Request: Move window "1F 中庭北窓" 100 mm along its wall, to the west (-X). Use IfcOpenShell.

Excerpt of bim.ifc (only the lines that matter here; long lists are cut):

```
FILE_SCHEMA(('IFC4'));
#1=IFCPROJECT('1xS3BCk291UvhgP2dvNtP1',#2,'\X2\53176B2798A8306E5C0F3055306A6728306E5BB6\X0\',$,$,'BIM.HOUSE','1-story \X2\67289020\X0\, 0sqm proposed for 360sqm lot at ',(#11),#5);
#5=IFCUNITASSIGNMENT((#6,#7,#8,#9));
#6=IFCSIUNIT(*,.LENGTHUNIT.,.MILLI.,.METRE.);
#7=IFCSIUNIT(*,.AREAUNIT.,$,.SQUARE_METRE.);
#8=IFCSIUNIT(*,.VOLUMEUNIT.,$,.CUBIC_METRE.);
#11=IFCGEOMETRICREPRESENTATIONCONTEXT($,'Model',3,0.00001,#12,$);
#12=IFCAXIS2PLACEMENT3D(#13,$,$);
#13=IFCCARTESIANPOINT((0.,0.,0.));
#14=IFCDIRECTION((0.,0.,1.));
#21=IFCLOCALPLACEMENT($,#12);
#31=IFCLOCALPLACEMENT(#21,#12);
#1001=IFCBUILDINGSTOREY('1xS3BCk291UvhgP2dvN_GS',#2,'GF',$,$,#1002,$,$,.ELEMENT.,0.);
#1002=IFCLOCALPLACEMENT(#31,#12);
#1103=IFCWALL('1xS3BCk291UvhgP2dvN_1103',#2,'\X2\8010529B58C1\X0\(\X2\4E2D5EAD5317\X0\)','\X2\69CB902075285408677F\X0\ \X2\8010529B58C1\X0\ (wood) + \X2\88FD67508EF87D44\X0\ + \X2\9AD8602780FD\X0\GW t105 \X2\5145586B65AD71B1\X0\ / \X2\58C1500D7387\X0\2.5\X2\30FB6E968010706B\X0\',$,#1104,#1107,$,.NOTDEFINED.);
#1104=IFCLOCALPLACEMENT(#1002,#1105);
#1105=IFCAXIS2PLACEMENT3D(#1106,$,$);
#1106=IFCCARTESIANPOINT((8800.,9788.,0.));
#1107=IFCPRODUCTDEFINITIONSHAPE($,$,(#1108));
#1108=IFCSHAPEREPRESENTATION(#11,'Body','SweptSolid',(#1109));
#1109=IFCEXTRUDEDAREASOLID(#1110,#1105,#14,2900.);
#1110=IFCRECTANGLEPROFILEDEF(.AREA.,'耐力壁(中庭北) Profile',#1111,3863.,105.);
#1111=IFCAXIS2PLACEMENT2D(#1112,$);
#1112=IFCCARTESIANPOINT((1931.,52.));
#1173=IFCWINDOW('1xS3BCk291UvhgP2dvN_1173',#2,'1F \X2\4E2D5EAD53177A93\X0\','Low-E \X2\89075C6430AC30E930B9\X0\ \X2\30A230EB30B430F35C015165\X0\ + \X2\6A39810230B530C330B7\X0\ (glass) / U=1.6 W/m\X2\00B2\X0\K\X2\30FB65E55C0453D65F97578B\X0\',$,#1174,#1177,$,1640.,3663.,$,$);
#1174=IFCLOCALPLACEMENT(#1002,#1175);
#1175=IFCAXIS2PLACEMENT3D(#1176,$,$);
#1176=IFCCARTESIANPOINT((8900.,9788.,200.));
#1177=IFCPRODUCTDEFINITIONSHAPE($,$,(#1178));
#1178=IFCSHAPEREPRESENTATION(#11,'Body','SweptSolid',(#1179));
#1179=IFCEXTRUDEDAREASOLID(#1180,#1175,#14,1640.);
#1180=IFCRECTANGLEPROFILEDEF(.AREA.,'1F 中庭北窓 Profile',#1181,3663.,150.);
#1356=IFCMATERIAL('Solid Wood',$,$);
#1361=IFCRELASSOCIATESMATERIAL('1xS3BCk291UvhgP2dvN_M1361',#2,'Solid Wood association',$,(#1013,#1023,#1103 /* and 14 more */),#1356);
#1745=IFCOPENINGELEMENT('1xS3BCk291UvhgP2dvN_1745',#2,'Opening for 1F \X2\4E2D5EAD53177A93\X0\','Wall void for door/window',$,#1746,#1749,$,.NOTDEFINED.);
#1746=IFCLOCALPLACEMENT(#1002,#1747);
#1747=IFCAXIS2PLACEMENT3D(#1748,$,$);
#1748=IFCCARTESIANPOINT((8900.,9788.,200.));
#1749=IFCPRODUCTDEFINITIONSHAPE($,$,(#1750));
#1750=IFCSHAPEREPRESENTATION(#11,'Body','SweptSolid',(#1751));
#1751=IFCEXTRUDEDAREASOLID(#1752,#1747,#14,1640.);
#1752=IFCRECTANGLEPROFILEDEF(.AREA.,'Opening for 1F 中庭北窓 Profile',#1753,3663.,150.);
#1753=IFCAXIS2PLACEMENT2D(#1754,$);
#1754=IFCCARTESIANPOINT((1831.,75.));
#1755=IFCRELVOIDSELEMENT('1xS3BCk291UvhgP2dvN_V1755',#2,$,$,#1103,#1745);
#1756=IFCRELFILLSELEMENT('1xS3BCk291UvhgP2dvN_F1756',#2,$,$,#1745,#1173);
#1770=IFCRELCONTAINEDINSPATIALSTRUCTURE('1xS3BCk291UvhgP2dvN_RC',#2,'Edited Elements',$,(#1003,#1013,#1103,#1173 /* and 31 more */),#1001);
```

```python
import ifcopenshell
import ifcopenshell.api.geometry
import ifcopenshell.util.placement
import ifcopenshell.util.unit

model = ifcopenshell.open("bim.ifc")
unit_scale = ifcopenshell.util.unit.calculate_unit_scale(model)

window = model.by_guid("1xS3BCk291UvhgP2dvN_1173")
opening = window.FillsVoids[0].RelatingOpeningElement
wall = opening.VoidsElements[0].RelatingBuildingElement

wall_matrix = ifcopenshell.util.placement.get_local_placement(wall.ObjectPlacement)
shift = wall_matrix[:3, 0] * -0.1 / unit_scale
before = ifcopenshell.util.placement.get_local_placement(window.ObjectPlacement)[:3, 3].copy()

# The window is not placed relative to its opening, so move both.
for product in (opening, window):
    matrix = ifcopenshell.util.placement.get_local_placement(product.ObjectPlacement)
    matrix[:3, 3] += shift
    ifcopenshell.api.geometry.edit_object_placement(model, product=product, matrix=matrix, is_si=False)

after = ifcopenshell.util.placement.get_local_placement(window.ObjectPlacement)[:3, 3]
print("window moved by", (after - before).round(3) + 0.0)

model.write("bim_rev.ifc")
```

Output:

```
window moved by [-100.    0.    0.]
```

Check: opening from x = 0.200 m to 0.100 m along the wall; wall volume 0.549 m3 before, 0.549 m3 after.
